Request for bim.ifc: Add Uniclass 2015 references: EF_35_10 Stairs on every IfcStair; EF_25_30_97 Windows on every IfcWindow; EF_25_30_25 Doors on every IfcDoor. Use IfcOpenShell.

First a look at what the model holds.

```python
import ifcopenshell

model = ifcopenshell.open("bim.ifc")
print(model.schema)
print("classifications:", [c.Name for c in model.by_type("IfcClassification")])
for ifc_class in ("IfcDoor", "IfcRoof", "IfcStair", "IfcWall", "IfcWindow"):
    print(ifc_class, len(model.by_type(ifc_class)))
```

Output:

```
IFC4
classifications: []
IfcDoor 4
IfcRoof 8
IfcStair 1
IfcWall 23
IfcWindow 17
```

```python
import ifcopenshell
import ifcopenshell.api.classification

model = ifcopenshell.open("bim.ifc")

system = ifcopenshell.api.classification.add_classification(model, classification="Uniclass 2015")

codes = {
    "IfcStair": ("EF_35_10", "Stairs"),
    "IfcWindow": ("EF_25_30_97", "Windows"),
    "IfcDoor": ("EF_25_30_25", "Doors"),
}
for ifc_class, (code, name) in codes.items():
    products = model.by_type(ifc_class)
    ifcopenshell.api.classification.add_reference(
        model, products=products, classification=system, identification=code, name=name
    )
    print(code, len(products))

model.write("bim_updated.ifc")
```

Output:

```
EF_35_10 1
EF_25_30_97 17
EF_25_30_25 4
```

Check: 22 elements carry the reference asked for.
